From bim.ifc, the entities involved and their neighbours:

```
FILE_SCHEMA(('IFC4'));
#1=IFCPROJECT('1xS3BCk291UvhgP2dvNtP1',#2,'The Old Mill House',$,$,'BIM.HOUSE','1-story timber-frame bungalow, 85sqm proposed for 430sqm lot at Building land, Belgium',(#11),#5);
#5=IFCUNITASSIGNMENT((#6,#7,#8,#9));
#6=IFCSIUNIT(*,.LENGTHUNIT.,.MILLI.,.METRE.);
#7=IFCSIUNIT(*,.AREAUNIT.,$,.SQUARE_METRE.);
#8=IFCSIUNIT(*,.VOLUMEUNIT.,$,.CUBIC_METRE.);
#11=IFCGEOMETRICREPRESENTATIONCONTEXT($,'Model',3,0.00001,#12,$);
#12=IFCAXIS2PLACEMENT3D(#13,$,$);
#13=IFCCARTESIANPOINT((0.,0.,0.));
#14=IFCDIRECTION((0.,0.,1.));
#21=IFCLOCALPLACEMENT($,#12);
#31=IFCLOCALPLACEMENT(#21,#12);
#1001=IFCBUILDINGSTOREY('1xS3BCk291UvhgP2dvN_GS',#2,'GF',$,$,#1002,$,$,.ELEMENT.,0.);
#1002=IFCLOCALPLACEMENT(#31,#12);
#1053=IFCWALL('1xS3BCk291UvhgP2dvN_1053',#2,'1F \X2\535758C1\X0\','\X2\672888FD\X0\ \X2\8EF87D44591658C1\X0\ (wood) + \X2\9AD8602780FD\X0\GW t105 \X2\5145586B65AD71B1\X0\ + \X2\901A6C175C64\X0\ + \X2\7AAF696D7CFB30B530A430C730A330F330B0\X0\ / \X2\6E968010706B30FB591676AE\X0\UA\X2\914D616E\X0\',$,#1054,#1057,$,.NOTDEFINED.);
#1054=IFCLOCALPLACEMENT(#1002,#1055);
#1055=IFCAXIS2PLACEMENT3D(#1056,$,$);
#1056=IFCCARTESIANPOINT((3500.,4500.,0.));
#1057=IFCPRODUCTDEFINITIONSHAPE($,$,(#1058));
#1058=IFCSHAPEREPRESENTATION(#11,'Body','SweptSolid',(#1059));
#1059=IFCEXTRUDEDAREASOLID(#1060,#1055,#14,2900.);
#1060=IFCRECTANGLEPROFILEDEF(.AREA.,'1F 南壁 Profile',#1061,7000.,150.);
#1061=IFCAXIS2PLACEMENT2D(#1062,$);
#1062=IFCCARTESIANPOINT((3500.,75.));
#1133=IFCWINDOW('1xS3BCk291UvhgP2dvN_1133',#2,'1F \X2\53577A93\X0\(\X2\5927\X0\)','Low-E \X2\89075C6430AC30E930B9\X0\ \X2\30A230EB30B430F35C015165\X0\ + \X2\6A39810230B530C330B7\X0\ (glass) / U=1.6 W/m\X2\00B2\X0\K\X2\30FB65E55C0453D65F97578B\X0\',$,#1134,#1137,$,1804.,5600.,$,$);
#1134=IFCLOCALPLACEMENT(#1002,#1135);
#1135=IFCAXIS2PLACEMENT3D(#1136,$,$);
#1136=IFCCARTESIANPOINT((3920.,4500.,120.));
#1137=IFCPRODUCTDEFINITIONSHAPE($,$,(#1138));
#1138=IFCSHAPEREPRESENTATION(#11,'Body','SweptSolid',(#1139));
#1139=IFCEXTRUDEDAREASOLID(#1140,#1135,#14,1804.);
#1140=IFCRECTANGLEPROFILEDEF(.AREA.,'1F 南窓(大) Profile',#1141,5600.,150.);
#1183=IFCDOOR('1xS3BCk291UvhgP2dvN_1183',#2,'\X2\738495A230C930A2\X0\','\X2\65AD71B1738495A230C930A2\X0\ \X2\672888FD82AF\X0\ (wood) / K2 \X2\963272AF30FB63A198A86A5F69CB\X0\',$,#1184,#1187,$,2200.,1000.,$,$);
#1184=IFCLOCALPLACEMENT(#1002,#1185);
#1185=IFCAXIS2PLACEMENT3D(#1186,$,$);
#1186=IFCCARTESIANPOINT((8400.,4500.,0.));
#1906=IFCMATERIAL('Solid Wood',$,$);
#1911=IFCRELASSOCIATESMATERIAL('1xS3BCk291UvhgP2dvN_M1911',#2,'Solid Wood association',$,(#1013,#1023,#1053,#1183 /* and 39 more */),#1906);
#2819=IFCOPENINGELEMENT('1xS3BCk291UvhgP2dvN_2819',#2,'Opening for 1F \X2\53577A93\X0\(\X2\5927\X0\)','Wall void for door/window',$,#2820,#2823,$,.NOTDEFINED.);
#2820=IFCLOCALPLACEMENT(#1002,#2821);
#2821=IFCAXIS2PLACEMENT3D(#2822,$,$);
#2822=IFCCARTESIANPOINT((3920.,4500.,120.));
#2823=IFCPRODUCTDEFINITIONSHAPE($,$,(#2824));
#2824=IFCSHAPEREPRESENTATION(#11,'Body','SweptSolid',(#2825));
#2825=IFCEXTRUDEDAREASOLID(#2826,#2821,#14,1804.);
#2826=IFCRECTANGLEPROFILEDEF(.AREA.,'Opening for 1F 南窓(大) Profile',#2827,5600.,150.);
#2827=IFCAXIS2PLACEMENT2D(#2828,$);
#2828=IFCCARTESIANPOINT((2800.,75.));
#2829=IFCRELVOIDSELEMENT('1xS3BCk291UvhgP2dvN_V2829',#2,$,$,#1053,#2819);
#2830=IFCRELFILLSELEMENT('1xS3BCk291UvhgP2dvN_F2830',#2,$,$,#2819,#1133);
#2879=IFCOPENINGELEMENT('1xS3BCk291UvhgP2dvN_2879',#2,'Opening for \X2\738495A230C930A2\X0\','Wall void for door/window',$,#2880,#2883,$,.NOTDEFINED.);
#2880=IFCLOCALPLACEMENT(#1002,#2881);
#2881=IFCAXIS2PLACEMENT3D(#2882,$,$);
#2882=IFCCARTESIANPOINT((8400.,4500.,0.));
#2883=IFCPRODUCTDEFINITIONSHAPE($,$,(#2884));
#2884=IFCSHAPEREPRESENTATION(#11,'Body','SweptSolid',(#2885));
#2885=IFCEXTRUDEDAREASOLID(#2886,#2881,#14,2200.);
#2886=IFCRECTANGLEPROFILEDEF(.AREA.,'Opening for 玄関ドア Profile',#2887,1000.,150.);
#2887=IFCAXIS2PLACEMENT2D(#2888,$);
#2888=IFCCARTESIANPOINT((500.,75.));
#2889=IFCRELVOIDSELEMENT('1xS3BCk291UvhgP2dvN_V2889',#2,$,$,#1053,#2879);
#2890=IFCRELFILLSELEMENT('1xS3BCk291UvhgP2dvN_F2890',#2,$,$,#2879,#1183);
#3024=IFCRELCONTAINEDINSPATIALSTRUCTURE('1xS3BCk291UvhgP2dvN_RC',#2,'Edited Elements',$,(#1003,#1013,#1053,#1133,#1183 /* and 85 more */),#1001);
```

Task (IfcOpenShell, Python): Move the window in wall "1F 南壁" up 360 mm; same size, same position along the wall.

```python
import numpy as np
import ifcopenshell
import ifcopenshell.api.geometry
import ifcopenshell.util.placement
import ifcopenshell.util.unit

model = ifcopenshell.open("bim.ifc")
unit_scale = ifcopenshell.util.unit.calculate_unit_scale(model)

window = model.by_guid("1xS3BCk291UvhgP2dvN_1133")
opening = window.FillsVoids[0].RelatingOpeningElement
dz = 360.0

shift = np.array([0.0, 0.0, dz])
# The window is not placed relative to its opening, so move both.
for product in (opening, window):
    matrix = ifcopenshell.util.placement.get_local_placement(product.ObjectPlacement)
    matrix[:3, 3] += shift
    ifcopenshell.api.geometry.edit_object_placement(model, product=product, matrix=matrix, is_si=False)

print(f"moved by {dz * unit_scale:+.3f} m")

model.write("bim_v2.ifc")
```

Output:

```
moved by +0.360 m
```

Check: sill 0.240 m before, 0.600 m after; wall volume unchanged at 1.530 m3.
